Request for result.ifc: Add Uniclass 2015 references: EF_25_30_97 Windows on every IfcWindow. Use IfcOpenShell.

First a look at what the model holds.

```python
import ifcopenshell

model = ifcopenshell.open("result.ifc")
print(model.schema)
print("classifications:", [c.Name for c in model.by_type("IfcClassification")])
for ifc_class in ("IfcDoor", "IfcRoof", "IfcStair", "IfcWall", "IfcWindow"):
    print(ifc_class, len(model.by_type(ifc_class)))
```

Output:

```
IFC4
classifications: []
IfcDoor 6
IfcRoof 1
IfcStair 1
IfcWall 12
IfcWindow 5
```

```python
import ifcopenshell
import ifcopenshell.api.classification

model = ifcopenshell.open("result.ifc")

system = ifcopenshell.api.classification.add_classification(model, classification="Uniclass 2015")

codes = {
    "IfcWindow": ("EF_25_30_97", "Windows"),
}
for ifc_class, (code, name) in codes.items():
    products = model.by_type(ifc_class)
    ifcopenshell.api.classification.add_reference(
        model, products=products, classification=system, identification=code, name=name
    )
    print(code, len(products))

model.write("result_updated.ifc")
```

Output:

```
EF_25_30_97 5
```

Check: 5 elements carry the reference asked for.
